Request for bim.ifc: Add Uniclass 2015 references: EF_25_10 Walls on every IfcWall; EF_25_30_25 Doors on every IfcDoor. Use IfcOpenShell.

First a look at what the model holds.

```python
import ifcopenshell

model = ifcopenshell.open("bim.ifc")
print(model.schema)
print("classifications:", [c.Name for c in model.by_type("IfcClassification")])
for ifc_class in ("IfcDoor", "IfcRoof", "IfcStair", "IfcWall", "IfcWindow"):
    print(ifc_class, len(model.by_type(ifc_class)))
```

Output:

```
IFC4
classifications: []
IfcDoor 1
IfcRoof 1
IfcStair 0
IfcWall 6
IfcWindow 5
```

```python
import ifcopenshell
import ifcopenshell.api.classification

model = ifcopenshell.open("bim.ifc")

system = ifcopenshell.api.classification.add_classification(model, classification="Uniclass 2015")

codes = {
    "IfcWall": ("EF_25_10", "Walls"),
    "IfcDoor": ("EF_25_30_25", "Doors"),
}
for ifc_class, (code, name) in codes.items():
    products = model.by_type(ifc_class)
    ifcopenshell.api.classification.add_reference(
        model, products=products, classification=system, identification=code, name=name
    )
    print(code, len(products))

model.write("bim_v2.ifc")
```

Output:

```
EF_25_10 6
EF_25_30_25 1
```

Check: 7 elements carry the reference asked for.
